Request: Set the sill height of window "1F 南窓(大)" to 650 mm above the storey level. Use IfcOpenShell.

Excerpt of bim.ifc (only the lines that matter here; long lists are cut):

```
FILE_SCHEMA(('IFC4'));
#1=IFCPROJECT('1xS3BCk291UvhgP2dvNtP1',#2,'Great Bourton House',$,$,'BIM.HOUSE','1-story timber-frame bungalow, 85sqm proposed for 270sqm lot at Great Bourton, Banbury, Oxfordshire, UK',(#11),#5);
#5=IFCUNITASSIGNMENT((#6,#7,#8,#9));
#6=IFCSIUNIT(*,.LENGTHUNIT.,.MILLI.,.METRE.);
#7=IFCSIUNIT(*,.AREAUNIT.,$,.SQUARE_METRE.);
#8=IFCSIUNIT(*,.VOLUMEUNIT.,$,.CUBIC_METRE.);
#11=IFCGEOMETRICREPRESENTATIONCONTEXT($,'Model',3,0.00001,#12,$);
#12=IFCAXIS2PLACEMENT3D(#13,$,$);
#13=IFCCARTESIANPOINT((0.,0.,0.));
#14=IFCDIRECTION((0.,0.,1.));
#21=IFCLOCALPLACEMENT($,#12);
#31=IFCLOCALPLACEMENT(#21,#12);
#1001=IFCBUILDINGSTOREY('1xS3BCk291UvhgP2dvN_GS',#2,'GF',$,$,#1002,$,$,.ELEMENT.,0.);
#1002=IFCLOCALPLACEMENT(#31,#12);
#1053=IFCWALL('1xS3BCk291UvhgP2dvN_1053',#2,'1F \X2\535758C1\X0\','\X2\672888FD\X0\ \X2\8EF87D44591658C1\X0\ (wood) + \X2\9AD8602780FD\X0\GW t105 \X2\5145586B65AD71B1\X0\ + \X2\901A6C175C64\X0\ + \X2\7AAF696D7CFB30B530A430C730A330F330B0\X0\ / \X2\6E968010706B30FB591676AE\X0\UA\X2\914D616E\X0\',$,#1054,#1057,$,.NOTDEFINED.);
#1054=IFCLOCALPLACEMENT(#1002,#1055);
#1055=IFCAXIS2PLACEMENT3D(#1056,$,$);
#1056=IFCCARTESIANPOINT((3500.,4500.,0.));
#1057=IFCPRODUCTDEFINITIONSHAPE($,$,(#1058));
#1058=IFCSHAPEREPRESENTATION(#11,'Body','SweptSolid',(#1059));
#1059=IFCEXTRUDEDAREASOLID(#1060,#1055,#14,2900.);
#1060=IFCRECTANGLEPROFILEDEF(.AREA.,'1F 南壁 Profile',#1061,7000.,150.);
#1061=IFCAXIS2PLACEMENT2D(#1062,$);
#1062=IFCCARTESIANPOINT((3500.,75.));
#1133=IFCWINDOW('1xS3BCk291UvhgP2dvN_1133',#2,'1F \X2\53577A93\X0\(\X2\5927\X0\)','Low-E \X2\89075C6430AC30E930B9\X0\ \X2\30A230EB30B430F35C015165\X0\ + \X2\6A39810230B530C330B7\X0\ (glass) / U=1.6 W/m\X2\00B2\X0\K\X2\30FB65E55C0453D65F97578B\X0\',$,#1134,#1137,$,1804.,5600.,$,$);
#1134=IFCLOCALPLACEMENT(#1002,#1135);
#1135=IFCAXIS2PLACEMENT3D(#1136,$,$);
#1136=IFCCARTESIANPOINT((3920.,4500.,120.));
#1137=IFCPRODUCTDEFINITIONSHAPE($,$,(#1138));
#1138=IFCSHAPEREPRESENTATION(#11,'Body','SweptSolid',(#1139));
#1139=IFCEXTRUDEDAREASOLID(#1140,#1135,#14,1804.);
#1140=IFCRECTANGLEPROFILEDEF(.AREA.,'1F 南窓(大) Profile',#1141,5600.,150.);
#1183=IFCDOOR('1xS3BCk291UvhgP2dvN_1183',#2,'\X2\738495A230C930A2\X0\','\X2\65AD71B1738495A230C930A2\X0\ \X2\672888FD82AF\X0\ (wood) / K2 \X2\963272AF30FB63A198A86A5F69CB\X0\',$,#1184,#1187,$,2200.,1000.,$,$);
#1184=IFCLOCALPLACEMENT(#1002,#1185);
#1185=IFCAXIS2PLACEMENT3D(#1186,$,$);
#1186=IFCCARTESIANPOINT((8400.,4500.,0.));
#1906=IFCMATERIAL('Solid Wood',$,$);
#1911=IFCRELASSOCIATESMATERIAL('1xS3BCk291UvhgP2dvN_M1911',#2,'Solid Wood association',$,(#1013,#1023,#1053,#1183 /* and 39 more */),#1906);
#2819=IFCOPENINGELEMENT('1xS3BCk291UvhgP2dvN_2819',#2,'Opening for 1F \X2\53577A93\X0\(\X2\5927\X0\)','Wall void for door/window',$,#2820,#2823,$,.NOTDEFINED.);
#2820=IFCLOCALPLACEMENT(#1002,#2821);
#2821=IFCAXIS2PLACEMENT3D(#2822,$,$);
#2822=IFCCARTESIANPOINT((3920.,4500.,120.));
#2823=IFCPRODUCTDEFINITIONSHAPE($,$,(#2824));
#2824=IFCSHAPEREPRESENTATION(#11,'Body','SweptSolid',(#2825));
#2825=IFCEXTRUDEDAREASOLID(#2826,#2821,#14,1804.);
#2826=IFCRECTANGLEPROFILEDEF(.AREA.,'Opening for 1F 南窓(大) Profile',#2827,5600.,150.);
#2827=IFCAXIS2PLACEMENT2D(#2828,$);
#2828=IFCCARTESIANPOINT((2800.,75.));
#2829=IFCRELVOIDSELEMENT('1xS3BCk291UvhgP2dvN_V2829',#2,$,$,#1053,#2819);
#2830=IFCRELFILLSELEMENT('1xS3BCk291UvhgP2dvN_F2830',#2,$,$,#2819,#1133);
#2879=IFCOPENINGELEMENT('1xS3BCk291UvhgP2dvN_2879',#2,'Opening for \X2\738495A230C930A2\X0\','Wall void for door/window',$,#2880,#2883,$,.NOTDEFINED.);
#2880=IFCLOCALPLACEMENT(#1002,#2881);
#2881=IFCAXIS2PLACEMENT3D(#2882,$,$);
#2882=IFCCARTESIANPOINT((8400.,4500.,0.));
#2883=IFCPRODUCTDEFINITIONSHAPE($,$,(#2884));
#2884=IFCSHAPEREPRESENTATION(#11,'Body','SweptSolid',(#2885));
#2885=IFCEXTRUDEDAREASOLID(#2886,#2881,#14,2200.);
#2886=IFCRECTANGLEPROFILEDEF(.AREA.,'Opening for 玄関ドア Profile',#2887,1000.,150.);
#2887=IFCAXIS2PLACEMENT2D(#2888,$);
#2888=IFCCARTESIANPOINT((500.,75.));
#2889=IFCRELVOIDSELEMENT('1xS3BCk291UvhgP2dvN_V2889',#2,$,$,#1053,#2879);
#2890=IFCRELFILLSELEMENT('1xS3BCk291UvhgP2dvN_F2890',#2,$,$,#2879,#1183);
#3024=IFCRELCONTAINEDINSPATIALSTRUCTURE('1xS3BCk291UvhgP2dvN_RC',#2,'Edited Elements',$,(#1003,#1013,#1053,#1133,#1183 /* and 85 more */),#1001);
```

```python
import numpy as np
import ifcopenshell
import ifcopenshell.api.geometry
import ifcopenshell.geom
import ifcopenshell.util.element
import ifcopenshell.util.placement
import ifcopenshell.util.shape
import ifcopenshell.util.unit

model = ifcopenshell.open("bim.ifc")
unit_scale = ifcopenshell.util.unit.calculate_unit_scale(model)

window = model.by_guid("1xS3BCk291UvhgP2dvN_1133")
opening = window.FillsVoids[0].RelatingOpeningElement
storey = ifcopenshell.util.element.get_container(window, ifc_class="IfcBuildingStorey")
level = ifcopenshell.util.placement.get_local_placement(storey.ObjectPlacement)[2, 3]

# The opening's origin need not be at the sill, so measure its lowest point.
shape = ifcopenshell.geom.create_shape(ifcopenshell.geom.settings(), opening)
bottom = ifcopenshell.util.shape.get_shape_bottom_elevation(shape, shape.geometry) / unit_scale
dz = level + 0.65 / unit_scale - bottom

shift = np.array([0.0, 0.0, dz])
# The window is not placed relative to its opening, so move both.
for product in (opening, window):
    matrix = ifcopenshell.util.placement.get_local_placement(product.ObjectPlacement)
    matrix[:3, 3] += shift
    ifcopenshell.api.geometry.edit_object_placement(model, product=product, matrix=matrix, is_si=False)

print(f"moved by {dz * unit_scale:+.3f} m")

model.write("bim_v2.ifc")
```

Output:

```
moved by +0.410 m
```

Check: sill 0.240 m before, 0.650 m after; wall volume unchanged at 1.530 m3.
